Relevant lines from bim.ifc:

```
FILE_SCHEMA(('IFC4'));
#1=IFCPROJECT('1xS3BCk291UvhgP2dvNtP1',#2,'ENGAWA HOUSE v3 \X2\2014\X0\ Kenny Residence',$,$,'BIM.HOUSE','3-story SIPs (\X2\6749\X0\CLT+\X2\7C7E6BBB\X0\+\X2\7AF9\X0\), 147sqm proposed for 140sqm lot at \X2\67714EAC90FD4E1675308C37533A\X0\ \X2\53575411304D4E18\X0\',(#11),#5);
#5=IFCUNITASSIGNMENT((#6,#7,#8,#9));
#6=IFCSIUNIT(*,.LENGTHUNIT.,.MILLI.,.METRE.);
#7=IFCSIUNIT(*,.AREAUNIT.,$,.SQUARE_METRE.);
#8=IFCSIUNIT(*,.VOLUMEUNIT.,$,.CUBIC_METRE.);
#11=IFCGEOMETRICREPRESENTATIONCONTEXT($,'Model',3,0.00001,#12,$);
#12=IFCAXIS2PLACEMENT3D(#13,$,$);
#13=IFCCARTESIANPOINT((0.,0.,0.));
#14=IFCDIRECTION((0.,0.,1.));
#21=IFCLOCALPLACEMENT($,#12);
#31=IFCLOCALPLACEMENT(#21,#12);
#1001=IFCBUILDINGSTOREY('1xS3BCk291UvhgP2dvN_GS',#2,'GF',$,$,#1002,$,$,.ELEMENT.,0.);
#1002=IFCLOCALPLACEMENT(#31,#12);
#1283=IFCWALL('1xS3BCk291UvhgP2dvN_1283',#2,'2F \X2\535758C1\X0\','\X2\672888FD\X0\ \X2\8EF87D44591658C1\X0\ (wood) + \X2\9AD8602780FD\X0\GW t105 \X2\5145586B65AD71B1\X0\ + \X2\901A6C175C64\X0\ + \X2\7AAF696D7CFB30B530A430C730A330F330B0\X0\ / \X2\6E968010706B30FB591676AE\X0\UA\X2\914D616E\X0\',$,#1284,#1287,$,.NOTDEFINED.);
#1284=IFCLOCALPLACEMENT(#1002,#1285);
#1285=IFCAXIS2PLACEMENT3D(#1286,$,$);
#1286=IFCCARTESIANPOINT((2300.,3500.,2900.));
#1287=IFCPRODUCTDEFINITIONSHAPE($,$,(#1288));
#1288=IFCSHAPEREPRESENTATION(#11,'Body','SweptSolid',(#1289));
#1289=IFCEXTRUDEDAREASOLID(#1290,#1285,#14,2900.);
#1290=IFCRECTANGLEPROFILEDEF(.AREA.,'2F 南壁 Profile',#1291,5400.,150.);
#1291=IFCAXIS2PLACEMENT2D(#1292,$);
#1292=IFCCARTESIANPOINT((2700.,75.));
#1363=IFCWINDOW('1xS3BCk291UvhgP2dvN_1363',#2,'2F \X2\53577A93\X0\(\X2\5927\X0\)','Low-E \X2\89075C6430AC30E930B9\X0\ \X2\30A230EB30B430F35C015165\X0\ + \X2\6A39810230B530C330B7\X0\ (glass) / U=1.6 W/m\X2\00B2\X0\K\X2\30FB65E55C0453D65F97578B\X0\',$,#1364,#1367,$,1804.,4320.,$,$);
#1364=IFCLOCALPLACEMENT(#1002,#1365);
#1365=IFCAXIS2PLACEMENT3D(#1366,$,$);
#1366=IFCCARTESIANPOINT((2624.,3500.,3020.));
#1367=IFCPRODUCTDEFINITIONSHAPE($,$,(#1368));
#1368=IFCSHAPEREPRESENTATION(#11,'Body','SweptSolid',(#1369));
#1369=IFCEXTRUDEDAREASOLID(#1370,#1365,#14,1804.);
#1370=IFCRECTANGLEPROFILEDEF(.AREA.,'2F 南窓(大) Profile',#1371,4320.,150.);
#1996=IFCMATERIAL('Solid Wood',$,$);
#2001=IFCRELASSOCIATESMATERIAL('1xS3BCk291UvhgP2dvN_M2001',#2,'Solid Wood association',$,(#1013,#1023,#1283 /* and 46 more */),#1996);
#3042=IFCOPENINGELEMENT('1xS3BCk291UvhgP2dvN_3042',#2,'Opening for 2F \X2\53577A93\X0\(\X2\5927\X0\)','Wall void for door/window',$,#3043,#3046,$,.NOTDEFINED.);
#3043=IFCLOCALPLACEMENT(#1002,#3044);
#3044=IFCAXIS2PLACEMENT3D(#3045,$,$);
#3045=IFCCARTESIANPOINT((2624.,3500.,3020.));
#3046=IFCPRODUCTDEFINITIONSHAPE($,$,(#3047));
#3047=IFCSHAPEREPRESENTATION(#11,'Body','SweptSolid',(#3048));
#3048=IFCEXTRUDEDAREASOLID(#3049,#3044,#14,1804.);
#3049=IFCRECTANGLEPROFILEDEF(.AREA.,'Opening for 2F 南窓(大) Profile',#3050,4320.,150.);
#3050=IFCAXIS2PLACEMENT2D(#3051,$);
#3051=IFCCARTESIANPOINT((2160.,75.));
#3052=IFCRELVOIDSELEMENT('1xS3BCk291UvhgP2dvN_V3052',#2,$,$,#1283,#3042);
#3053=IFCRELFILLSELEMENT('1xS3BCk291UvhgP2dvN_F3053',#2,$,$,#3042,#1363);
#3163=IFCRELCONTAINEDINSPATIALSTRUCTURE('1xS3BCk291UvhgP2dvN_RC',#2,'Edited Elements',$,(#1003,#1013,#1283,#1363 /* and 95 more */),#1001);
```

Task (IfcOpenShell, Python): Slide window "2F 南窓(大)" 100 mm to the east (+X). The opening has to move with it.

```python
import ifcopenshell
import ifcopenshell.api.geometry
import ifcopenshell.util.placement
import ifcopenshell.util.unit

model = ifcopenshell.open("bim.ifc")
unit_scale = ifcopenshell.util.unit.calculate_unit_scale(model)

window = model.by_guid("1xS3BCk291UvhgP2dvN_1363")
opening = window.FillsVoids[0].RelatingOpeningElement
wall = opening.VoidsElements[0].RelatingBuildingElement

wall_matrix = ifcopenshell.util.placement.get_local_placement(wall.ObjectPlacement)
shift = wall_matrix[:3, 0] * 0.1 / unit_scale
before = ifcopenshell.util.placement.get_local_placement(window.ObjectPlacement)[:3, 3].copy()

# The window is not placed relative to its opening, so move both.
for product in (opening, window):
    matrix = ifcopenshell.util.placement.get_local_placement(product.ObjectPlacement)
    matrix[:3, 3] += shift
    ifcopenshell.api.geometry.edit_object_placement(model, product=product, matrix=matrix, is_si=False)

after = ifcopenshell.util.placement.get_local_placement(window.ObjectPlacement)[:3, 3]
print("window moved by", (after - before).round(3) + 0.0)

model.write("bim_edited.ifc")
```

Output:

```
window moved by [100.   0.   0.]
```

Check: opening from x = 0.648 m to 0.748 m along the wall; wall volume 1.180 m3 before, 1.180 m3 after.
